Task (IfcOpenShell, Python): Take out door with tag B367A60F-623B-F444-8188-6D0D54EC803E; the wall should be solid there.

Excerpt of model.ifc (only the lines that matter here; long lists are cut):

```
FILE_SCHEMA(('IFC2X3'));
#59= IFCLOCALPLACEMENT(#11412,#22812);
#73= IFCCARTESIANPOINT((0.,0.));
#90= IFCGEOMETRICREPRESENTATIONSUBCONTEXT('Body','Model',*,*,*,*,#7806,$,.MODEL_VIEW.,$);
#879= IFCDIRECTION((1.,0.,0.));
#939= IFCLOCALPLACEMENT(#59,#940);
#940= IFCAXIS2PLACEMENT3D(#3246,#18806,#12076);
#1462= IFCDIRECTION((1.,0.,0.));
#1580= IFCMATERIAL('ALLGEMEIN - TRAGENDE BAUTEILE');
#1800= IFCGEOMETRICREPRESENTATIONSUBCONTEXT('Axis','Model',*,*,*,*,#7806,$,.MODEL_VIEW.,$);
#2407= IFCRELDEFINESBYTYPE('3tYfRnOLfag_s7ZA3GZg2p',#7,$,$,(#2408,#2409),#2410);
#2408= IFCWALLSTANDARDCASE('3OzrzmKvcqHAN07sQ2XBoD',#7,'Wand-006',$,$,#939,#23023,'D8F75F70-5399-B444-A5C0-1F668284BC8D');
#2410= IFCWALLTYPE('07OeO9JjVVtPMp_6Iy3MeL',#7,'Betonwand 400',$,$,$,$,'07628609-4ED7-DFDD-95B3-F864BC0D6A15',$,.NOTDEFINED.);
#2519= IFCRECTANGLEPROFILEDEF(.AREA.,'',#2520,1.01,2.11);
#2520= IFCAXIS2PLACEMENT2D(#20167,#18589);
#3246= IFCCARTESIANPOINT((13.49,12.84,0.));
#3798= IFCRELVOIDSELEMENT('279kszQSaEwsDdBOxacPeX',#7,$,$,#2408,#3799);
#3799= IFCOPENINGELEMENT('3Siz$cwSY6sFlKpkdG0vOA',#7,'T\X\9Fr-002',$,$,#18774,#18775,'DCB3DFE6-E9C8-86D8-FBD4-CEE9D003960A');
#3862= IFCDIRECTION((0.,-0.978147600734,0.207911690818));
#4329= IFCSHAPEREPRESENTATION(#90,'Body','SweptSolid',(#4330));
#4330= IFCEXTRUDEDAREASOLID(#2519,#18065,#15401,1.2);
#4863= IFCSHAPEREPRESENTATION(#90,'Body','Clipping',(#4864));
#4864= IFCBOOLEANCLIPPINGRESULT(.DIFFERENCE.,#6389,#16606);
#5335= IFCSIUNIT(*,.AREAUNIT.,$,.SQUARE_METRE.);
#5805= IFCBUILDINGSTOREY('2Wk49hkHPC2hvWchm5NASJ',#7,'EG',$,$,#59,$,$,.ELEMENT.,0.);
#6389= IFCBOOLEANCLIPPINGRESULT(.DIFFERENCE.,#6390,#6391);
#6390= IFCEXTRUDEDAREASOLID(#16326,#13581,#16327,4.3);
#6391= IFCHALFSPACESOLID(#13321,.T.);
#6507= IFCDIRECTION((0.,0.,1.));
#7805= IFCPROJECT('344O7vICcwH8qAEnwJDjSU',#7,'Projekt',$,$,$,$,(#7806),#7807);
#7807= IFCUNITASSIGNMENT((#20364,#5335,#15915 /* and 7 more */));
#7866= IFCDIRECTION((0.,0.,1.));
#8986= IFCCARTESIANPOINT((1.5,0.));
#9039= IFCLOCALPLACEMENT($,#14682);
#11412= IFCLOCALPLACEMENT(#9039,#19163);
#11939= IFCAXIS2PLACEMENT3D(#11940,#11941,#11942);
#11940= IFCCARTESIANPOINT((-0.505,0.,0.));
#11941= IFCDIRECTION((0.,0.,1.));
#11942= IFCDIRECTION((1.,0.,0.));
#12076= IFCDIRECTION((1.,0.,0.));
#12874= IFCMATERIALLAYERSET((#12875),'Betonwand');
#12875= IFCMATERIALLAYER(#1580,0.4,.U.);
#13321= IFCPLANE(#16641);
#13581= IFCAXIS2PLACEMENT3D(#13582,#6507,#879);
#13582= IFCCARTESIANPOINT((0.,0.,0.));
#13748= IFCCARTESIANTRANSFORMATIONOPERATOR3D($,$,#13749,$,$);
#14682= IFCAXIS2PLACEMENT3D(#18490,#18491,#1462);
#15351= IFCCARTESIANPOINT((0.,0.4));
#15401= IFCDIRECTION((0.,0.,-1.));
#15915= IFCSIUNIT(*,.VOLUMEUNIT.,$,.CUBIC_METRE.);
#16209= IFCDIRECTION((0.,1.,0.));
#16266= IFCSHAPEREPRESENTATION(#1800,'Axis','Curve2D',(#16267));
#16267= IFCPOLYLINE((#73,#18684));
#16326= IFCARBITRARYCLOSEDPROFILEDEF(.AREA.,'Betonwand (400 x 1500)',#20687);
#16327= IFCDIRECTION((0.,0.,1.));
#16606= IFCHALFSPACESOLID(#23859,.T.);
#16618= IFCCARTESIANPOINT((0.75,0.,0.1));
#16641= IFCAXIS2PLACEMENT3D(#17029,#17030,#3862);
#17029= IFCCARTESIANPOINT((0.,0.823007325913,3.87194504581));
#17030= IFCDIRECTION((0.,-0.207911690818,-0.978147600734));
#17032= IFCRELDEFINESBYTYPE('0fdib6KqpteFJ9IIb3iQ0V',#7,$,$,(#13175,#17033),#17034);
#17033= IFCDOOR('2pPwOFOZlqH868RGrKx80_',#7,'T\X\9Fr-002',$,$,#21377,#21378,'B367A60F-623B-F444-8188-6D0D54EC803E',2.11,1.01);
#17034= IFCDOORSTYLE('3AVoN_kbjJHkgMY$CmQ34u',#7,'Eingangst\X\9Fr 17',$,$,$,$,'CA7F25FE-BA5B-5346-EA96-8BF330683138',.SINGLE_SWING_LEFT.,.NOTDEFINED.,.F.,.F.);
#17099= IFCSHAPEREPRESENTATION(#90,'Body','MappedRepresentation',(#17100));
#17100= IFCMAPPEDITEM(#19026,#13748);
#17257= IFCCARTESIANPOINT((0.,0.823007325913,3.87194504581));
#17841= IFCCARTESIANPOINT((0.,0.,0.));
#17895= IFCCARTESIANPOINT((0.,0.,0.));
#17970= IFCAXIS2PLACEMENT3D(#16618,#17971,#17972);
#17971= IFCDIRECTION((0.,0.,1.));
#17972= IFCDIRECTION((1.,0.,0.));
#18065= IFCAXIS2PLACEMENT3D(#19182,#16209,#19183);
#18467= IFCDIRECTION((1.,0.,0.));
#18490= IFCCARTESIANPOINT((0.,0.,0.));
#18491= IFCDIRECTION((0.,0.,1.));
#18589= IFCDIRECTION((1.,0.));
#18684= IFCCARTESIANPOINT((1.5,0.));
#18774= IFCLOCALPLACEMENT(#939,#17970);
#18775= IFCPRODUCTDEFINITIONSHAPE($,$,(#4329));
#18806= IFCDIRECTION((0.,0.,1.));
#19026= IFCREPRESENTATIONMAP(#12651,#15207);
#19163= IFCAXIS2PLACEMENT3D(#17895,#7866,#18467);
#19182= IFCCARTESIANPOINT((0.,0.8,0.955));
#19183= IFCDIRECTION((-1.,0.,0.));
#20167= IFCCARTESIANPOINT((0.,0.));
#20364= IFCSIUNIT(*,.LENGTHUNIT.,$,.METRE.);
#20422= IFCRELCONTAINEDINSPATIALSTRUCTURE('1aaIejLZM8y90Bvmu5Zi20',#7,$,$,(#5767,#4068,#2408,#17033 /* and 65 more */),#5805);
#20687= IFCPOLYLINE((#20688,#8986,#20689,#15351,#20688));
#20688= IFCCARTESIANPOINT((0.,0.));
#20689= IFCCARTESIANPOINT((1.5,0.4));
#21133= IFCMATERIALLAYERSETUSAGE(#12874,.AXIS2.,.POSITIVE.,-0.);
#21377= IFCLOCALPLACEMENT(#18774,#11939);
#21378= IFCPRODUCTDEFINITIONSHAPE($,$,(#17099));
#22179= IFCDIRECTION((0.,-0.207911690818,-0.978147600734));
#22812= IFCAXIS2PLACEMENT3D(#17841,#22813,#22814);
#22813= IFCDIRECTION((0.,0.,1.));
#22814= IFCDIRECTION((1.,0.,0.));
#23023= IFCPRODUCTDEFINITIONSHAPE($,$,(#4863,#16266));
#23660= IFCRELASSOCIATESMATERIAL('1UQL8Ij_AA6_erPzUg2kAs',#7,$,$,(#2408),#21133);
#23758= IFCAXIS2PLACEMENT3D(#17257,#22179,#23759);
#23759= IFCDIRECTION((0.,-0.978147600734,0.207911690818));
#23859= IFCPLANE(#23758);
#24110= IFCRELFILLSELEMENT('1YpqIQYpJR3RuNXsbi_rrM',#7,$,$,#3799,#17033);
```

```python
import ifcopenshell
import ifcopenshell.api.feature
import ifcopenshell.api.root
import ifcopenshell.geom
import ifcopenshell.util.shape

model = ifcopenshell.open("model.ifc")
settings = ifcopenshell.geom.settings()


def volume(element):
    """Net volume in cubic metres, openings subtracted."""
    shape = ifcopenshell.geom.create_shape(settings, element)
    return ifcopenshell.util.shape.get_volume(shape.geometry)


door = model.by_guid("2pPwOFOZlqH868RGrKx80_")
opening = door.FillsVoids[0].RelatingOpeningElement
wall = opening.VoidsElements[0].RelatingBuildingElement
before = volume(wall)

ifcopenshell.api.root.remove_product(model, product=door)
ifcopenshell.api.feature.remove_feature(model, feature=opening)

after = volume(wall)

print(f"wall volume {before:.3f} -> {after:.3f} m3")

model.write("model_v2.ifc")
```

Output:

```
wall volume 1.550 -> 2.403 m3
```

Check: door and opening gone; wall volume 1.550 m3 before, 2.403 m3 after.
